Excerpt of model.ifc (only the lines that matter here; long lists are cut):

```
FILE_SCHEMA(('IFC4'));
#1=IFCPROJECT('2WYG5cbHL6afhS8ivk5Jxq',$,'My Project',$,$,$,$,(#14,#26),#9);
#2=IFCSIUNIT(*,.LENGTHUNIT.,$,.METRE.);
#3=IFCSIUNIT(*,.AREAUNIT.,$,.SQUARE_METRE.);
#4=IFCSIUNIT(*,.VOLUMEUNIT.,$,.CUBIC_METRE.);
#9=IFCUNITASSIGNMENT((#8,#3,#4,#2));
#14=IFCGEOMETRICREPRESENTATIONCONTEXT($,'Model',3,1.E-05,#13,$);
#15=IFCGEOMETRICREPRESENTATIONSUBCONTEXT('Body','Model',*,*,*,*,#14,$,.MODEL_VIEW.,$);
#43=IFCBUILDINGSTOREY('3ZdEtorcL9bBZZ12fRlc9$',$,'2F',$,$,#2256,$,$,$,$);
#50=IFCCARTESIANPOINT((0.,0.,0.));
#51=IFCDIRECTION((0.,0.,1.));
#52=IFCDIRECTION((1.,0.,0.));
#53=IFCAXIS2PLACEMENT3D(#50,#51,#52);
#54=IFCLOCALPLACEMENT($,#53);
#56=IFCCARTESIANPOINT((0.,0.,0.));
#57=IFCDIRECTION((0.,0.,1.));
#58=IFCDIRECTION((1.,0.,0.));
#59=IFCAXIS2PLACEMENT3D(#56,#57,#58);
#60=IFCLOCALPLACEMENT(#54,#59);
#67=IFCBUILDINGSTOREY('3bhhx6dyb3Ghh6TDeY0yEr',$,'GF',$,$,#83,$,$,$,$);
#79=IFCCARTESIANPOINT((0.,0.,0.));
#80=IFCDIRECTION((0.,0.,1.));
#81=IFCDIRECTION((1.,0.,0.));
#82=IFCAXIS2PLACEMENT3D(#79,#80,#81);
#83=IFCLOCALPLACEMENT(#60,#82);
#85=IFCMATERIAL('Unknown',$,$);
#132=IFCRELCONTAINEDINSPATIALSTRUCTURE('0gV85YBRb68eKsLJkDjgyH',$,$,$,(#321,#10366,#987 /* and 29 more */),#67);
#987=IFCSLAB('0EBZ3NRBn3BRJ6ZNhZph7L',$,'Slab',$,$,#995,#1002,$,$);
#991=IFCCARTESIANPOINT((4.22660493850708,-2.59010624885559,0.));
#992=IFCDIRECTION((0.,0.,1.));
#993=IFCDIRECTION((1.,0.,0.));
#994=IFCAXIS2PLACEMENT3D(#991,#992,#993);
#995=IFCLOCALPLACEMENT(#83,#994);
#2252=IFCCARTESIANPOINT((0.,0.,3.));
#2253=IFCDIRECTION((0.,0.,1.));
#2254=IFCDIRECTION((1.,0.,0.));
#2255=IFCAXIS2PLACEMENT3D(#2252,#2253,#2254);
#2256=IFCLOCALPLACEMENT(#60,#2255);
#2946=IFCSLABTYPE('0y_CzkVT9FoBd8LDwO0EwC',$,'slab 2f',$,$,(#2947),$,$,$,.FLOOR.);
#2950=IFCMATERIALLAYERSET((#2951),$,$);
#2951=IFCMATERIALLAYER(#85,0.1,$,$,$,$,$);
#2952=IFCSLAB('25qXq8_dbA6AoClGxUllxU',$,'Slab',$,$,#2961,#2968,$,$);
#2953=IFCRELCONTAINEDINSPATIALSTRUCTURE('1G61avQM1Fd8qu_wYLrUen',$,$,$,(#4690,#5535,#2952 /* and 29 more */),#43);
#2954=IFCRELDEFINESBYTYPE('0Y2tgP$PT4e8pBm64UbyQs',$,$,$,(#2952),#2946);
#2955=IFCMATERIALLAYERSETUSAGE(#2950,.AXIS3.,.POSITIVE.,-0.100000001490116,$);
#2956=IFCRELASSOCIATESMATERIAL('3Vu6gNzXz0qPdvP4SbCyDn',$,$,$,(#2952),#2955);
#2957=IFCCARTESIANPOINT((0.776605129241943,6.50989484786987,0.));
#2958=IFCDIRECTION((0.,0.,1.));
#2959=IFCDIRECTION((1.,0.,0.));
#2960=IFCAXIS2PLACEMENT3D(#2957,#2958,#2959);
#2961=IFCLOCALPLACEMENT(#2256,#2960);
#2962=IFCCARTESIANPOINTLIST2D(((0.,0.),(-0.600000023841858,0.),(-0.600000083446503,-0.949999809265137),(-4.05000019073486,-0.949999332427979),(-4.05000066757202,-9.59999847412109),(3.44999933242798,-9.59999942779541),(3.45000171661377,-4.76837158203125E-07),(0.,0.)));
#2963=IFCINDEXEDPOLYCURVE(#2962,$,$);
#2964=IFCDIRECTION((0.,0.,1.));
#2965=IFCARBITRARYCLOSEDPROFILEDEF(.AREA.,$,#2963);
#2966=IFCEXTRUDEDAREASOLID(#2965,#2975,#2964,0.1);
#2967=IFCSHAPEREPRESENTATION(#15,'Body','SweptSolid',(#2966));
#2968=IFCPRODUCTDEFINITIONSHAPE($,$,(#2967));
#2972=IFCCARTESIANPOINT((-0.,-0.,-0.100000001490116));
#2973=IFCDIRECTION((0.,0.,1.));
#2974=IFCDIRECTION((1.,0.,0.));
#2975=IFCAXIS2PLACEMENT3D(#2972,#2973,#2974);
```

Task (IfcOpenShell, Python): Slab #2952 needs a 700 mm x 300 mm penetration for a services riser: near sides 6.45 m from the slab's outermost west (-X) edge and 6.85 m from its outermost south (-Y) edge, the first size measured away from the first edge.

```python
import numpy as np
import ifcopenshell
import ifcopenshell.api.feature
import ifcopenshell.api.geometry
import ifcopenshell.api.root
import ifcopenshell.geom
import ifcopenshell.util.placement
import ifcopenshell.util.representation
import ifcopenshell.util.shape
import ifcopenshell.util.unit

model = ifcopenshell.open("model.ifc")
unit_scale = ifcopenshell.util.unit.calculate_unit_scale(model)
settings = ifcopenshell.geom.settings()


def volume(element):
    """Net volume in cubic metres, openings subtracted."""
    shape = ifcopenshell.geom.create_shape(settings, element)
    return ifcopenshell.util.shape.get_volume(shape.geometry)


slab = model.by_guid("25qXq8_dbA6AoClGxUllxU")
before = volume(slab)

# Extent in the slab's own axes, in metres. The edges named are its -X and -Y sides.
slab_shape = ifcopenshell.geom.create_shape(settings, slab)
vertices = ifcopenshell.util.shape.get_vertices(slab_shape.geometry)
x_min, y_min, bottom = vertices.min(axis=0)
top = vertices[:, 2].max()

opening = ifcopenshell.api.root.create_entity(model, ifc_class="IfcOpeningElement", name="Services riser opening", predefined_type="OPENING")
context = ifcopenshell.util.representation.get_context(model, "Model", "Body", "MODEL_VIEW")
width, depth = 0.7, 0.3
outline = [(0.0, 0.0), (width, 0.0), (width, depth), (0.0, depth), (0.0, 0.0)]
# Overshoot both faces by 50 mm so the cut is clean.
shape = ifcopenshell.api.geometry.add_slab_representation(
    model, context=context, depth=top - bottom + 0.1, polyline=outline
)
ifcopenshell.api.geometry.assign_representation(model, product=opening, representation=shape)

matrix = ifcopenshell.util.placement.get_local_placement(slab.ObjectPlacement)
matrix[:, 3] = matrix @ np.append(np.array([x_min + 6.45, y_min + 6.85, bottom - 0.05]) / unit_scale, 1.0)
ifcopenshell.api.geometry.edit_object_placement(model, product=opening, matrix=matrix, is_si=False)
ifcopenshell.api.feature.add_feature(model, feature=opening, element=slab)

after = volume(slab)

print(f"slab volume {before:.3f} -> {after:.3f} m3")

model.write("model_updated.ifc")
```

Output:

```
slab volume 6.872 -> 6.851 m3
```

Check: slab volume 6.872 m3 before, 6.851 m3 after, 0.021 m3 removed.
